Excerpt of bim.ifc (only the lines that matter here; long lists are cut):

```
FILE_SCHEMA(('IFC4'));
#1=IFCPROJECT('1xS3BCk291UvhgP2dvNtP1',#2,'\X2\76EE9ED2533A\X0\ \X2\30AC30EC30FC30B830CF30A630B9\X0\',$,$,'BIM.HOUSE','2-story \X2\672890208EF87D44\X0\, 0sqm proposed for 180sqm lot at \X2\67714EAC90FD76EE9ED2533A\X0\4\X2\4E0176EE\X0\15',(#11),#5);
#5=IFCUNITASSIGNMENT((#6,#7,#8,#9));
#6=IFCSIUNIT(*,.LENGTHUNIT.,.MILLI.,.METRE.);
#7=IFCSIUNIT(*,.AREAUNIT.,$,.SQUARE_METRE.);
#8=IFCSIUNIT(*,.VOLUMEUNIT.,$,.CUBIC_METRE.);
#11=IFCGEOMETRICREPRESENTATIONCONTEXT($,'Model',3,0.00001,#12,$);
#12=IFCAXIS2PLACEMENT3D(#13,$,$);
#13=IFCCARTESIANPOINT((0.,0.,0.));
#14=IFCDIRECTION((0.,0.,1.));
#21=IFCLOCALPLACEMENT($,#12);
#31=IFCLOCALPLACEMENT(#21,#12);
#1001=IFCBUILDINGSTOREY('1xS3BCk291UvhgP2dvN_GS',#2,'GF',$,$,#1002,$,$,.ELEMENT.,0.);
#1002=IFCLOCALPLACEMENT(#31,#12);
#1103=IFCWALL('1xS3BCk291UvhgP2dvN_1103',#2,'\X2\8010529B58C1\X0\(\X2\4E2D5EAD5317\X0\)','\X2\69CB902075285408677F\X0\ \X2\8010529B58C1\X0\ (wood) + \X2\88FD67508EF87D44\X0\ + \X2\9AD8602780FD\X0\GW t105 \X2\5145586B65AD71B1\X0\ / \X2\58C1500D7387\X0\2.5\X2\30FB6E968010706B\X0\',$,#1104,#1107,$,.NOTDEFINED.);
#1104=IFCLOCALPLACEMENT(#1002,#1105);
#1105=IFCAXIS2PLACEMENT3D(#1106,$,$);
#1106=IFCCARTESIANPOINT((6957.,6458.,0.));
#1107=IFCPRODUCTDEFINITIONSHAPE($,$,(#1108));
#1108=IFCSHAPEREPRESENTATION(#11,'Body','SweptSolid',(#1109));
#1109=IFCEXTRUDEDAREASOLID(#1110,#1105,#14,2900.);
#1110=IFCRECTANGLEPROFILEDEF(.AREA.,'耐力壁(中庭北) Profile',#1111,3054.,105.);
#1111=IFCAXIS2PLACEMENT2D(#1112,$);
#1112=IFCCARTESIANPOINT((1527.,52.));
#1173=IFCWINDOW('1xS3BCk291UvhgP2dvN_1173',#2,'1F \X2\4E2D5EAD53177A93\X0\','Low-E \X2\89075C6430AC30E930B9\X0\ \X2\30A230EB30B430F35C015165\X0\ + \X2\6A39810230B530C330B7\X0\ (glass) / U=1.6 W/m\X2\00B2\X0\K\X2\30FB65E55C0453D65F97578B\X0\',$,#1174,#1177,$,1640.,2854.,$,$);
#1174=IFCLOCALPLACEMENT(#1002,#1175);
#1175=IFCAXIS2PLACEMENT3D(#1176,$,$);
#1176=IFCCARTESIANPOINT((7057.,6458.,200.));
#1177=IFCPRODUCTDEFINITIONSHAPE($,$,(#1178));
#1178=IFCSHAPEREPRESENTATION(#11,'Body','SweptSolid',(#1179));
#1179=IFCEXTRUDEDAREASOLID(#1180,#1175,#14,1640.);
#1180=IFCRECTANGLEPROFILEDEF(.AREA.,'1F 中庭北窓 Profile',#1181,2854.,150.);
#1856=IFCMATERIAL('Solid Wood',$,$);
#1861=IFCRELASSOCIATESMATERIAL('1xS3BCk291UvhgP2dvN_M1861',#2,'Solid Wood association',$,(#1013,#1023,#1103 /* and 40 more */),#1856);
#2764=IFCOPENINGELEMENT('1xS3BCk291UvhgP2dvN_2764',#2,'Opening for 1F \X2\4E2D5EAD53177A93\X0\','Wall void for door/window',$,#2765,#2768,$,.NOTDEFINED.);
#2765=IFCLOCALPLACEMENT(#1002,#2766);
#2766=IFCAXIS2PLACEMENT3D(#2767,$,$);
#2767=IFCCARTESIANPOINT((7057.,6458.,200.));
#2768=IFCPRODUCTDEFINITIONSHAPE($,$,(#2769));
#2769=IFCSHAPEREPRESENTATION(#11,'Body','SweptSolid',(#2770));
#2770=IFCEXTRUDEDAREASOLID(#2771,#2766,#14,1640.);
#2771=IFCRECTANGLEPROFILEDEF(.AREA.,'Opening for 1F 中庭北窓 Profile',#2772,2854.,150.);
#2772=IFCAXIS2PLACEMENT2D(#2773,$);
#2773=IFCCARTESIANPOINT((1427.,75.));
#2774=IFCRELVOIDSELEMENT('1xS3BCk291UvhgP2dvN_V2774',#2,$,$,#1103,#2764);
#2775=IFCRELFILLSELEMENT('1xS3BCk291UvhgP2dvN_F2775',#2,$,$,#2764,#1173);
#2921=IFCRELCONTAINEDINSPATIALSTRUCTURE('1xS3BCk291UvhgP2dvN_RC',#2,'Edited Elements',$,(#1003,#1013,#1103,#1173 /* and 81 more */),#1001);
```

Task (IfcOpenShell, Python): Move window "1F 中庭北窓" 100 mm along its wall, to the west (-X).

```python
import ifcopenshell
import ifcopenshell.api.geometry
import ifcopenshell.util.placement

model = ifcopenshell.open("bim.ifc")

window = model.by_id(1173)
opening = window.FillsVoids[0].RelatingOpeningElement
wall = opening.VoidsElements[0].RelatingBuildingElement

wall_matrix = ifcopenshell.util.placement.get_local_placement(wall.ObjectPlacement)
shift = wall_matrix[:3, 0] * -100.0
before = ifcopenshell.util.placement.get_local_placement(window.ObjectPlacement)[:3, 3].copy()

# The window is not placed relative to its opening, so move both.
for product in (opening, window):
    matrix = ifcopenshell.util.placement.get_local_placement(product.ObjectPlacement)
    matrix[:3, 3] += shift
    ifcopenshell.api.geometry.edit_object_placement(model, product=product, matrix=matrix, is_si=False)

after = ifcopenshell.util.placement.get_local_placement(window.ObjectPlacement)[:3, 3]
print("window moved by", (after - before).round(3) + 0.0)

model.write("bim_updated.ifc")
```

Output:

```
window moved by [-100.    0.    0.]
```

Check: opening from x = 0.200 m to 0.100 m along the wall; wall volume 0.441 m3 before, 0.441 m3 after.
